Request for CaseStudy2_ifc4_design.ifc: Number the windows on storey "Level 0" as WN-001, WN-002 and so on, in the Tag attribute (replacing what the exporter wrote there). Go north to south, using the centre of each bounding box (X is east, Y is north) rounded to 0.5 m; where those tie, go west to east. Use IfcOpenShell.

First a look at what the model holds.

```python
import ifcopenshell
import ifcopenshell.util.element
import ifcopenshell.util.placement

model = ifcopenshell.open("CaseStudy2_ifc4_design.ifc")
print(model.schema)
storey = next(s for s in model.by_type("IfcBuildingStorey") if s.Name == "Level 0")
windows = [e for e in ifcopenshell.util.element.get_decomposition(storey) if e.is_a("IfcWindow")]
for e in sorted(windows, key=lambda e: e.id()):
    origin = ifcopenshell.util.placement.get_local_placement(e.ObjectPlacement)[:3, 3]
    print(e.id(), e.Tag, e.Name, origin.round(2) + 0.0, sep=" | ")
```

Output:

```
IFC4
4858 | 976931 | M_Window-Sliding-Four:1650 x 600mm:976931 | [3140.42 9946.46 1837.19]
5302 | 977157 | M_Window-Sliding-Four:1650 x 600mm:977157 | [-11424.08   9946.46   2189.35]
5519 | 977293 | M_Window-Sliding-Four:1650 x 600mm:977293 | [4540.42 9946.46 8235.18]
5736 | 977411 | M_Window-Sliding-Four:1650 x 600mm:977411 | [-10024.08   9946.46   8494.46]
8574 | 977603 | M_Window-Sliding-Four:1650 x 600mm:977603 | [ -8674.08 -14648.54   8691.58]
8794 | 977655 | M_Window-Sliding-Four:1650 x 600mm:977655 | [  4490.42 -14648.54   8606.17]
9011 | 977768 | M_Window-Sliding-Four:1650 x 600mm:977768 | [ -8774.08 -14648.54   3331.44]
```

```python
import ifcopenshell
import ifcopenshell.geom
import ifcopenshell.util.element
import ifcopenshell.util.shape

model = ifcopenshell.open("CaseStudy2_ifc4_design.ifc")
settings = ifcopenshell.geom.settings()
settings.set("use-world-coords", True)


def centre(element):
    shape = ifcopenshell.geom.create_shape(settings, element)
    return ifcopenshell.util.shape.get_bbox_centroid(shape.geometry)


storey = next(s for s in model.by_type("IfcBuildingStorey") if s.Name == "Level 0")
windows = [e for e in ifcopenshell.util.element.get_decomposition(storey) if e.is_a("IfcWindow")]

# Insertion points can sit at a corner or the storey origin, so sort by the geometry (in metres).
centres = {e: centre(e) for e in windows}
windows.sort(key=lambda e: (-round(centres[e][1] / 0.5), centres[e][0]))

for i, e in enumerate(windows, start=1):
    number = f"WN-0{i:02d}"
    e.Tag = number
    print(e.id(), number)

model.write("CaseStudy2_ifc4_design_edited.ifc")
```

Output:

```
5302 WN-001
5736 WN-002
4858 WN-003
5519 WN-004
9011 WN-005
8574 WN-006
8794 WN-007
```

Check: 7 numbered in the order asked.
